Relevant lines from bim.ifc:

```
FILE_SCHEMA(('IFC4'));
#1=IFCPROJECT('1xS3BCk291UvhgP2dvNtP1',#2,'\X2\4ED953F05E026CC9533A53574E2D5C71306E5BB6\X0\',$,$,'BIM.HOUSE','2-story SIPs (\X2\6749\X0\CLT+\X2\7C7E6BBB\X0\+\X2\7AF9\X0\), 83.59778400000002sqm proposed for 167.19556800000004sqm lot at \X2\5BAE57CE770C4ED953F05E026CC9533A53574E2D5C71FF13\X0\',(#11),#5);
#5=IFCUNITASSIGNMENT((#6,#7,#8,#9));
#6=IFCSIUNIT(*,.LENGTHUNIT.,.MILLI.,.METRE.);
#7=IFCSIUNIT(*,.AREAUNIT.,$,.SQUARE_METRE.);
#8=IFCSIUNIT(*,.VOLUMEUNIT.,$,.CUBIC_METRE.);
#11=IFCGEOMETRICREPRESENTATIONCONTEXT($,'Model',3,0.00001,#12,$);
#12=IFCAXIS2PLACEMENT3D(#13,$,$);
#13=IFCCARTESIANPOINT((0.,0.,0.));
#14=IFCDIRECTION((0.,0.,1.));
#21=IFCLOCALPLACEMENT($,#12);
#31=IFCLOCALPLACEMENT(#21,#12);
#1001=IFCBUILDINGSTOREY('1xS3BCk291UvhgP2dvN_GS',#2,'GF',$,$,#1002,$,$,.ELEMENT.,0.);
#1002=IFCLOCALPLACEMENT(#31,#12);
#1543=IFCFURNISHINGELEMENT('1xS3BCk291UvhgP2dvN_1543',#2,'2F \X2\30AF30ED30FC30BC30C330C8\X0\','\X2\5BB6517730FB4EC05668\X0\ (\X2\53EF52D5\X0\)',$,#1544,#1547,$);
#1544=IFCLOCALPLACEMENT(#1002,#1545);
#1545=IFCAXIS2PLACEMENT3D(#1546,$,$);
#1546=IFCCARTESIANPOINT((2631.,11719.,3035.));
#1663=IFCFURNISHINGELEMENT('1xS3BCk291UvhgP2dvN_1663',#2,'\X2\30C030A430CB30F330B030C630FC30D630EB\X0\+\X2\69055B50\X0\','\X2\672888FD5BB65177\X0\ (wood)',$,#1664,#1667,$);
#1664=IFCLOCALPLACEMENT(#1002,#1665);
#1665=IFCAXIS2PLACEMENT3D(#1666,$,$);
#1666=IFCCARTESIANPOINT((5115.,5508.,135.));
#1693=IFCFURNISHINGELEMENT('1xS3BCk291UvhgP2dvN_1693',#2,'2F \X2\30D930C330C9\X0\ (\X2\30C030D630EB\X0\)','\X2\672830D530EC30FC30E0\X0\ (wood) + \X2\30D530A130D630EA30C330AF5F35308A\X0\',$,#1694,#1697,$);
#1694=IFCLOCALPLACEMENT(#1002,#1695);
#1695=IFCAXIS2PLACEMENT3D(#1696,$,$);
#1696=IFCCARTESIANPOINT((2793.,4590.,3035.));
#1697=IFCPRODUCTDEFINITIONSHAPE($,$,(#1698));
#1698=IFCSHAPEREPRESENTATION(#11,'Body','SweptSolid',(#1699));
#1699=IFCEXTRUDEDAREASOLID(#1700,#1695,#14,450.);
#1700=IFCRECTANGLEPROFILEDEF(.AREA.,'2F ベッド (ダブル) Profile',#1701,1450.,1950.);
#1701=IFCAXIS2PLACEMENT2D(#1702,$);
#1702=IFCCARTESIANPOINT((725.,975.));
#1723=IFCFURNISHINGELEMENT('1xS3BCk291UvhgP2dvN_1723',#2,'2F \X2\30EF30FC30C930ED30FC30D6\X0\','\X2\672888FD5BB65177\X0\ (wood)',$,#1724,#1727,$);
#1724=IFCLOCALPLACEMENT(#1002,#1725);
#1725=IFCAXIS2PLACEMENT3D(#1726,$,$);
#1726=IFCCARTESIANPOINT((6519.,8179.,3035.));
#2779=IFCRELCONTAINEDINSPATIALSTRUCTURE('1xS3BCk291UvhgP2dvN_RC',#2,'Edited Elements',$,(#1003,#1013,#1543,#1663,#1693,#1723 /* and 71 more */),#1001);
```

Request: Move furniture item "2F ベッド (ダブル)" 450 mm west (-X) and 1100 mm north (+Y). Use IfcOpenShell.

```python
import ifcopenshell
import ifcopenshell.api.geometry
import ifcopenshell.util.placement
import ifcopenshell.util.unit

model = ifcopenshell.open("bim.ifc")
unit_scale = ifcopenshell.util.unit.calculate_unit_scale(model)

item = model.by_id(1693)
matrix = ifcopenshell.util.placement.get_local_placement(item.ObjectPlacement)
matrix[0, 3] -= 0.45 / unit_scale
matrix[1, 3] += 1.1 / unit_scale
ifcopenshell.api.geometry.edit_object_placement(model, product=item, matrix=matrix, is_si=False)

print(ifcopenshell.util.placement.get_local_placement(item.ObjectPlacement).round(3) + 0.0)

model.write("bim_edited.ifc")
```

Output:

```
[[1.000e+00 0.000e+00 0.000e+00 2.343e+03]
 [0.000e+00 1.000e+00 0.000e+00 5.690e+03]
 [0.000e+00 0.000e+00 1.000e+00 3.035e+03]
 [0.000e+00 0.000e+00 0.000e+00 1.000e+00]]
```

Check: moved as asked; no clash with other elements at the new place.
